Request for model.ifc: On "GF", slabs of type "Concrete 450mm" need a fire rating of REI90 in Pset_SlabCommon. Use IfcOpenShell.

First a look at what the model holds.

```python
import ifcopenshell
import ifcopenshell.util.element

model = ifcopenshell.open("model.ifc")
print(model.schema)
storey = next(s for s in model.by_type("IfcBuildingStorey") if s.Name == "GF")
slabs = [e for e in ifcopenshell.util.element.get_decomposition(storey) if e.is_a("IfcSlab")]
seen = {}
for e in slabs:
    element_type = ifcopenshell.util.element.get_type(e)
    key = (element_type.Name if element_type != e and element_type else None, ifcopenshell.util.element.get_pset(e, "Pset_SlabCommon", "FireRating"))
    seen[key] = seen.get(key, 0) + 1
for (name, value), count in sorted(seen.items(), key=str):
    print(count, "x", name, "|", value)
```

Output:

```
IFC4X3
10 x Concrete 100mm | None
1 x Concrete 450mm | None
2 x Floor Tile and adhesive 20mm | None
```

```python
import ifcopenshell
import ifcopenshell.api.pset
import ifcopenshell.util.element

model = ifcopenshell.open("model.ifc")

storey = next(s for s in model.by_type("IfcBuildingStorey") if s.Name == "GF")
slabs = [e for e in ifcopenshell.util.element.get_decomposition(storey) if e.is_a("IfcSlab")]

count = 0
for e in slabs:
    element_type = ifcopenshell.util.element.get_type(e)
    if element_type in (None, e) or element_type.Name != "Concrete 450mm":
        continue
    # add_pset returns the element's existing set when there is one.
    pset = ifcopenshell.api.pset.add_pset(model, product=e, name="Pset_SlabCommon")
    ifcopenshell.api.pset.edit_pset(model, pset=pset, properties={"FireRating": "REI90"})
    count += 1

print(count, "slabs updated")

model.write("model-out.ifc")
```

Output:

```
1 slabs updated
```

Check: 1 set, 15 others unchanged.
